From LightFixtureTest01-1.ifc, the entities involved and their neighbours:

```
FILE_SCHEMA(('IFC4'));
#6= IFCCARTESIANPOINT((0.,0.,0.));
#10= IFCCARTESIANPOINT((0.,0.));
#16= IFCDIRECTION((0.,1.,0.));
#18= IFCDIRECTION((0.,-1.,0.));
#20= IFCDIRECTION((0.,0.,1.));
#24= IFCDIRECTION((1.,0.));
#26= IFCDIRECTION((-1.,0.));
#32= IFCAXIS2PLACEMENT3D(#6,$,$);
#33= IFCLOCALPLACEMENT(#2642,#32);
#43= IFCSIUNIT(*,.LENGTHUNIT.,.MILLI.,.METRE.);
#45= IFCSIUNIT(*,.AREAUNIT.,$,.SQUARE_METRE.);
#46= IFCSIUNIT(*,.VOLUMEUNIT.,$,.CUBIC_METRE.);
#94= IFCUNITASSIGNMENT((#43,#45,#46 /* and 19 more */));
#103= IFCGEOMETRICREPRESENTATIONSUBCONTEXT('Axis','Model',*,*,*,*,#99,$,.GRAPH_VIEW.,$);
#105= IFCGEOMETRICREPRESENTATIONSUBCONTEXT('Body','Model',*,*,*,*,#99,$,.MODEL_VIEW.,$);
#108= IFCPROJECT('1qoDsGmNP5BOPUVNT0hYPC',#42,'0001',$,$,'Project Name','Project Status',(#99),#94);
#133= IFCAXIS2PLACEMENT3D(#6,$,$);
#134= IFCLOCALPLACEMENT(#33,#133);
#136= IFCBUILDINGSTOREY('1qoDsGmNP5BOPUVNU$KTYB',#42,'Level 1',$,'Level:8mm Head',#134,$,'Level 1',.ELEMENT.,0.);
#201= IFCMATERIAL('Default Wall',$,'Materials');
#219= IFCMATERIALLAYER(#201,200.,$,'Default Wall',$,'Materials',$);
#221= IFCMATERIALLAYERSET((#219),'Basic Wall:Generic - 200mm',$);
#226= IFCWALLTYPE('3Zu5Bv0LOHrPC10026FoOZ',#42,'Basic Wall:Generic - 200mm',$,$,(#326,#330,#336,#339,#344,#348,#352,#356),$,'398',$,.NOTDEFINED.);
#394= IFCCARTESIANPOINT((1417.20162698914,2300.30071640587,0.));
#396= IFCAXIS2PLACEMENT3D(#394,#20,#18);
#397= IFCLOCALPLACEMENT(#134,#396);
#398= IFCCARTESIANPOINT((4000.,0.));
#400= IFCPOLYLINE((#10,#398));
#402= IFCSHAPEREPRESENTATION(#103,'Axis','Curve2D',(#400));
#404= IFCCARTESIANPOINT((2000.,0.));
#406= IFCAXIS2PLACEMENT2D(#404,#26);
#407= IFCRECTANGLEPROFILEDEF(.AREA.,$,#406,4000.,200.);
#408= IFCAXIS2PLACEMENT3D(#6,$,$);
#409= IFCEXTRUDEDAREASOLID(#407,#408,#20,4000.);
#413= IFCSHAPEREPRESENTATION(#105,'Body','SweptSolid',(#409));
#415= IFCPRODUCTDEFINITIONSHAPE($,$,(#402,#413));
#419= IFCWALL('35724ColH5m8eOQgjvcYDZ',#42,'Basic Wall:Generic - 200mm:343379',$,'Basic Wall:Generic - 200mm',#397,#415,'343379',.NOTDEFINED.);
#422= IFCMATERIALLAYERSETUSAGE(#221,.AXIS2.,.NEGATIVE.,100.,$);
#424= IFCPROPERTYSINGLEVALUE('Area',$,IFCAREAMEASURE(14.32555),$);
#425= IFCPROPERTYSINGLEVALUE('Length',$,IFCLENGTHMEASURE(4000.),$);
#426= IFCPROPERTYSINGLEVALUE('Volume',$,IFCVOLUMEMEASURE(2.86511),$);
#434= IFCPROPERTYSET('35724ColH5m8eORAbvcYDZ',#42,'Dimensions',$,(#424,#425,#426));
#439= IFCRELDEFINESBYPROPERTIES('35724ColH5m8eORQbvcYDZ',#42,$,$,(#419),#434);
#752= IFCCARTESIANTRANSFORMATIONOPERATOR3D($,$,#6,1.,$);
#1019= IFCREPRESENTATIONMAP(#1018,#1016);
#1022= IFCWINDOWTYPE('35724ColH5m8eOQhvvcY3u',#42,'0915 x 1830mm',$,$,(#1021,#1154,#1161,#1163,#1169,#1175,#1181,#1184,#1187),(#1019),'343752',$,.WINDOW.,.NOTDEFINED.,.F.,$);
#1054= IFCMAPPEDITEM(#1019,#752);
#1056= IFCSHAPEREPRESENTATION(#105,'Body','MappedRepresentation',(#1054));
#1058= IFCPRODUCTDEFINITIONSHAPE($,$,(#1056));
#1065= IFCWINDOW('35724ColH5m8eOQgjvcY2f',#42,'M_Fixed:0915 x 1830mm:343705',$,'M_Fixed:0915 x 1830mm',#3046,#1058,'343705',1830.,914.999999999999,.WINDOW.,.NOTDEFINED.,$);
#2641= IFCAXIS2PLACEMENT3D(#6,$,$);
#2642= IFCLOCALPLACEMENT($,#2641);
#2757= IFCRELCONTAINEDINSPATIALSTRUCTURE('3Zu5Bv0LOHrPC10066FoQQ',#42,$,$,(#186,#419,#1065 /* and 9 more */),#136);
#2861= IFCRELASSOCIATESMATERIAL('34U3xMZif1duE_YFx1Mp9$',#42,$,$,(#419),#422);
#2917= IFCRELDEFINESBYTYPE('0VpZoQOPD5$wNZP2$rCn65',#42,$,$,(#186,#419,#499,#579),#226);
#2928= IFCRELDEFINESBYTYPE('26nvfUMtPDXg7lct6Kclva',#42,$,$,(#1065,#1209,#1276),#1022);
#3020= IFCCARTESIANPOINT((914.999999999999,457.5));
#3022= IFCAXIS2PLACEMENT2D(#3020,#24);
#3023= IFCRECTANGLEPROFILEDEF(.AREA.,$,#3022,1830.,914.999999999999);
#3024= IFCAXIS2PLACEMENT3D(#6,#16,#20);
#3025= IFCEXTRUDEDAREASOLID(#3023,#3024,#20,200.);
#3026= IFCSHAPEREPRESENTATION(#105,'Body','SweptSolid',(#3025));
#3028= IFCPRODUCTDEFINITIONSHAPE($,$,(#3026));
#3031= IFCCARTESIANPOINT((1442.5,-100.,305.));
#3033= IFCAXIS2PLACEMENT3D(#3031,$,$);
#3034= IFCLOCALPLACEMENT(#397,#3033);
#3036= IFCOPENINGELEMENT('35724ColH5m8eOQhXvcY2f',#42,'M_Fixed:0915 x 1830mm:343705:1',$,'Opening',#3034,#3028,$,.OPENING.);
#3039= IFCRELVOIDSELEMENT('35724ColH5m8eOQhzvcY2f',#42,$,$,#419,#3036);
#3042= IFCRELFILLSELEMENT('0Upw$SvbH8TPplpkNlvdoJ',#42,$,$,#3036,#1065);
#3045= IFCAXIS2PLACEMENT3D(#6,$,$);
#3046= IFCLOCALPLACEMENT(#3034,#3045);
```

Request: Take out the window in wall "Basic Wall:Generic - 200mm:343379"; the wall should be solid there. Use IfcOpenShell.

```python
import ifcopenshell
import ifcopenshell.api.feature
import ifcopenshell.api.pset
import ifcopenshell.api.root
import ifcopenshell.geom
import ifcopenshell.util.element
import ifcopenshell.util.shape
import ifcopenshell.util.unit

model = ifcopenshell.open("LightFixtureTest01-1.ifc")
area_scale = ifcopenshell.util.unit.calculate_unit_scale(model, "AREAUNIT")
volume_scale = ifcopenshell.util.unit.calculate_unit_scale(model, "VOLUMEUNIT")
settings = ifcopenshell.geom.settings()


def volume(element):
    """Net volume in cubic metres, openings subtracted."""
    shape = ifcopenshell.geom.create_shape(settings, element)
    return ifcopenshell.util.shape.get_volume(shape.geometry)


window = model.by_id(1065)
opening = window.FillsVoids[0].RelatingOpeningElement
wall = opening.VoidsElements[0].RelatingBuildingElement
before = volume(wall)

ifcopenshell.api.root.remove_product(model, product=window)
ifcopenshell.api.feature.remove_feature(model, feature=opening)

after = volume(wall)
thickness = 0.2  # wall thickness in metres

# Update the wall's stored quantities.
pset = model.by_id(ifcopenshell.util.element.get_pset(wall, "Dimensions", should_inherit=False)["id"])
ifcopenshell.api.pset.edit_pset(model, pset=pset, properties={
    "Area": model.create_entity("IfcAreaMeasure", after / thickness / area_scale),
    "Volume": model.create_entity("IfcVolumeMeasure", after / volume_scale),
})

print(f"wall volume {before:.3f} -> {after:.3f} m3")

model.write("LightFixtureTest01-1_rev.ifc")
```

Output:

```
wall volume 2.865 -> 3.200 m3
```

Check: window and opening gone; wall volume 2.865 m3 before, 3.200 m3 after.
